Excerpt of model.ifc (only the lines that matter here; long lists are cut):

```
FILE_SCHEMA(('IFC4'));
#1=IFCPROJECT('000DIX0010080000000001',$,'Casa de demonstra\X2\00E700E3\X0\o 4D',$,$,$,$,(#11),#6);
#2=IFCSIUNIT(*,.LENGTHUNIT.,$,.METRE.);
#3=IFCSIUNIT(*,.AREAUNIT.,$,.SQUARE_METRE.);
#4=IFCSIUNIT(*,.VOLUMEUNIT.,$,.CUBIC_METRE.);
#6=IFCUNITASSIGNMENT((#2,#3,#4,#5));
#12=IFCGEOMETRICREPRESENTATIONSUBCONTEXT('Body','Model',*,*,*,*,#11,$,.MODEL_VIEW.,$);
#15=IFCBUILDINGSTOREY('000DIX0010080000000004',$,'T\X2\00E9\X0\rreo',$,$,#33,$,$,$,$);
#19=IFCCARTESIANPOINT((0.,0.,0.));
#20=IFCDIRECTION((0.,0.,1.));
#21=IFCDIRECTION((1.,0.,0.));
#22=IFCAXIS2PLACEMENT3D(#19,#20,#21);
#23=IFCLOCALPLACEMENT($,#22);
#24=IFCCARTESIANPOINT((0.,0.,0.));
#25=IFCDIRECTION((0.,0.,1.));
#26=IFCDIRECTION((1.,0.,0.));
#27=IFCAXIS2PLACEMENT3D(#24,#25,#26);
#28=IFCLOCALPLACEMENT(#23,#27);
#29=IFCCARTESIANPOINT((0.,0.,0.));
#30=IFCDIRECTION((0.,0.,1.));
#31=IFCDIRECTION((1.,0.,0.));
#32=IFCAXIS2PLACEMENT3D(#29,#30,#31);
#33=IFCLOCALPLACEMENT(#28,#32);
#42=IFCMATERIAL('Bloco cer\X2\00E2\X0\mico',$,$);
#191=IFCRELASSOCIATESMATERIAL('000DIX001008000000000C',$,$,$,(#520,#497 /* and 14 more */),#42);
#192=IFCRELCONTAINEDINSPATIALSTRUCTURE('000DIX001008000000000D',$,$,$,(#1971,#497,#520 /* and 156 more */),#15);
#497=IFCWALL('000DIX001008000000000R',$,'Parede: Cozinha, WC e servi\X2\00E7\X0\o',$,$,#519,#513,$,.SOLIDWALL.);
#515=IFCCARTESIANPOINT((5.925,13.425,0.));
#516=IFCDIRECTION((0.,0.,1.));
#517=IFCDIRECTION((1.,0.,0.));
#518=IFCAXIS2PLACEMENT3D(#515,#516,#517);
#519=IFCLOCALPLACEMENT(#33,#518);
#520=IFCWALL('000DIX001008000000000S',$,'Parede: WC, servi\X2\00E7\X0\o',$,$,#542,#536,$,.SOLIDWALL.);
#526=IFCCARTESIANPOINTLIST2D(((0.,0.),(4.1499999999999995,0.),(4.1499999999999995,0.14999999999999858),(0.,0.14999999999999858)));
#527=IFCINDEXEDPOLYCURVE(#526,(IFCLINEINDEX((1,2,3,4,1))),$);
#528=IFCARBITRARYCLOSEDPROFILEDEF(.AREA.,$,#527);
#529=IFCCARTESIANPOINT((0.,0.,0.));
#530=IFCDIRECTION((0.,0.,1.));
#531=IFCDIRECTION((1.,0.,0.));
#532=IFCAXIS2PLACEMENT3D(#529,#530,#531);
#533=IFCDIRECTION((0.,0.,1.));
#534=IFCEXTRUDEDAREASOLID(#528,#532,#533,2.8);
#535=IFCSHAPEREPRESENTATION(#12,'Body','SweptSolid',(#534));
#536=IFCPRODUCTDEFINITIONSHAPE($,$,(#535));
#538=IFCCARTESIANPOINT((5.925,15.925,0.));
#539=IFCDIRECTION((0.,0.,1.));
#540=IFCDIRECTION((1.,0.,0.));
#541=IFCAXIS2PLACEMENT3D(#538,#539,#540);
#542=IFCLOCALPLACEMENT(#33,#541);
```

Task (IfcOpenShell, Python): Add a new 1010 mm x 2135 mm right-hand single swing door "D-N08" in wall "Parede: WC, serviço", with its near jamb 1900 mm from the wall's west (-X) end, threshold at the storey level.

```python
import numpy as np
import ifcopenshell
import ifcopenshell.api.feature
import ifcopenshell.api.geometry
import ifcopenshell.api.root
import ifcopenshell.api.spatial
import ifcopenshell.geom
import ifcopenshell.util.element
import ifcopenshell.util.placement
import ifcopenshell.util.representation
import ifcopenshell.util.shape
import ifcopenshell.util.unit

model = ifcopenshell.open("model.ifc")
unit_scale = ifcopenshell.util.unit.calculate_unit_scale(model)
settings = ifcopenshell.geom.settings()


def volume(element):
    """Net volume in cubic metres, openings subtracted."""
    shape = ifcopenshell.geom.create_shape(settings, element)
    return ifcopenshell.util.shape.get_volume(shape.geometry)


wall = model.by_guid("000DIX001008000000000S")
storey = ifcopenshell.util.element.get_container(wall, ifc_class="IfcBuildingStorey")
context = ifcopenshell.util.representation.get_context(model, "Model", "Body", "MODEL_VIEW")
before = volume(wall)

width, height, from_end, sill = 1.01, 2.135, 1.9, 0.0  # metres

# The wall runs along its own X axis, and the end named is its -X end.
wall_shape = ifcopenshell.geom.create_shape(settings, wall)
x, y, z = ifcopenshell.util.shape.get_vertices(wall_shape.geometry).T
start = x.min() + from_end
face, thickness = float(y.min()), float(y.max() - y.min())
wall_matrix = ifcopenshell.util.placement.get_local_placement(wall.ObjectPlacement)
level = ifcopenshell.util.placement.get_local_placement(storey.ObjectPlacement)[2, 3]


def in_wall(x, y):
    """Placement at x, y metres in the wall's axes, at sill height."""
    matrix = wall_matrix.copy()
    matrix[:, 3] = wall_matrix @ np.array([x / unit_scale, y / unit_scale, 0.0, 1.0])
    matrix[2, 3] = level + sill / unit_scale
    return matrix


# Opening: a box that overshoots both wall faces by 50 mm.
opening = ifcopenshell.api.root.create_entity(model, ifc_class="IfcOpeningElement", predefined_type="OPENING")
box = ifcopenshell.api.geometry.add_wall_representation(
    model, context=context, length=width, height=height, thickness=thickness + 0.1
)
ifcopenshell.api.geometry.assign_representation(model, product=opening, representation=box)
ifcopenshell.api.geometry.edit_object_placement(model, product=opening, matrix=in_wall(start, face - 0.05), is_si=False)
ifcopenshell.api.feature.add_feature(model, feature=opening, element=wall)

door = ifcopenshell.api.root.create_entity(model, ifc_class="IfcDoor", name="D-N08", predefined_type="DOOR")
door.OverallWidth, door.OverallHeight = width / unit_scale, height / unit_scale
door.OperationType = "SINGLE_SWING_RIGHT"
body = ifcopenshell.api.geometry.add_door_representation(
    model,
    context=context,
    overall_width=door.OverallWidth,
    overall_height=door.OverallHeight,
    operation_type="SINGLE_SWING_RIGHT",
    lining_properties={"LiningDepth": thickness / unit_scale, "ThresholdDepth": thickness / unit_scale},
)
ifcopenshell.api.geometry.assign_representation(model, product=door, representation=body)
ifcopenshell.api.spatial.assign_container(model, products=[door], relating_structure=storey)
ifcopenshell.api.feature.add_filling(model, opening=opening, element=door)

# The lining spans the wall, so the door starts at the wall face.
ifcopenshell.api.geometry.edit_object_placement(model, product=door, matrix=in_wall(start, face), is_si=False)

after = volume(wall)

print(f"wall volume {before:.3f} -> {after:.3f} m3")

model.write("model_rev.ifc")
```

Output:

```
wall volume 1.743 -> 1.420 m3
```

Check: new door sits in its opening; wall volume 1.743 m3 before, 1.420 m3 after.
